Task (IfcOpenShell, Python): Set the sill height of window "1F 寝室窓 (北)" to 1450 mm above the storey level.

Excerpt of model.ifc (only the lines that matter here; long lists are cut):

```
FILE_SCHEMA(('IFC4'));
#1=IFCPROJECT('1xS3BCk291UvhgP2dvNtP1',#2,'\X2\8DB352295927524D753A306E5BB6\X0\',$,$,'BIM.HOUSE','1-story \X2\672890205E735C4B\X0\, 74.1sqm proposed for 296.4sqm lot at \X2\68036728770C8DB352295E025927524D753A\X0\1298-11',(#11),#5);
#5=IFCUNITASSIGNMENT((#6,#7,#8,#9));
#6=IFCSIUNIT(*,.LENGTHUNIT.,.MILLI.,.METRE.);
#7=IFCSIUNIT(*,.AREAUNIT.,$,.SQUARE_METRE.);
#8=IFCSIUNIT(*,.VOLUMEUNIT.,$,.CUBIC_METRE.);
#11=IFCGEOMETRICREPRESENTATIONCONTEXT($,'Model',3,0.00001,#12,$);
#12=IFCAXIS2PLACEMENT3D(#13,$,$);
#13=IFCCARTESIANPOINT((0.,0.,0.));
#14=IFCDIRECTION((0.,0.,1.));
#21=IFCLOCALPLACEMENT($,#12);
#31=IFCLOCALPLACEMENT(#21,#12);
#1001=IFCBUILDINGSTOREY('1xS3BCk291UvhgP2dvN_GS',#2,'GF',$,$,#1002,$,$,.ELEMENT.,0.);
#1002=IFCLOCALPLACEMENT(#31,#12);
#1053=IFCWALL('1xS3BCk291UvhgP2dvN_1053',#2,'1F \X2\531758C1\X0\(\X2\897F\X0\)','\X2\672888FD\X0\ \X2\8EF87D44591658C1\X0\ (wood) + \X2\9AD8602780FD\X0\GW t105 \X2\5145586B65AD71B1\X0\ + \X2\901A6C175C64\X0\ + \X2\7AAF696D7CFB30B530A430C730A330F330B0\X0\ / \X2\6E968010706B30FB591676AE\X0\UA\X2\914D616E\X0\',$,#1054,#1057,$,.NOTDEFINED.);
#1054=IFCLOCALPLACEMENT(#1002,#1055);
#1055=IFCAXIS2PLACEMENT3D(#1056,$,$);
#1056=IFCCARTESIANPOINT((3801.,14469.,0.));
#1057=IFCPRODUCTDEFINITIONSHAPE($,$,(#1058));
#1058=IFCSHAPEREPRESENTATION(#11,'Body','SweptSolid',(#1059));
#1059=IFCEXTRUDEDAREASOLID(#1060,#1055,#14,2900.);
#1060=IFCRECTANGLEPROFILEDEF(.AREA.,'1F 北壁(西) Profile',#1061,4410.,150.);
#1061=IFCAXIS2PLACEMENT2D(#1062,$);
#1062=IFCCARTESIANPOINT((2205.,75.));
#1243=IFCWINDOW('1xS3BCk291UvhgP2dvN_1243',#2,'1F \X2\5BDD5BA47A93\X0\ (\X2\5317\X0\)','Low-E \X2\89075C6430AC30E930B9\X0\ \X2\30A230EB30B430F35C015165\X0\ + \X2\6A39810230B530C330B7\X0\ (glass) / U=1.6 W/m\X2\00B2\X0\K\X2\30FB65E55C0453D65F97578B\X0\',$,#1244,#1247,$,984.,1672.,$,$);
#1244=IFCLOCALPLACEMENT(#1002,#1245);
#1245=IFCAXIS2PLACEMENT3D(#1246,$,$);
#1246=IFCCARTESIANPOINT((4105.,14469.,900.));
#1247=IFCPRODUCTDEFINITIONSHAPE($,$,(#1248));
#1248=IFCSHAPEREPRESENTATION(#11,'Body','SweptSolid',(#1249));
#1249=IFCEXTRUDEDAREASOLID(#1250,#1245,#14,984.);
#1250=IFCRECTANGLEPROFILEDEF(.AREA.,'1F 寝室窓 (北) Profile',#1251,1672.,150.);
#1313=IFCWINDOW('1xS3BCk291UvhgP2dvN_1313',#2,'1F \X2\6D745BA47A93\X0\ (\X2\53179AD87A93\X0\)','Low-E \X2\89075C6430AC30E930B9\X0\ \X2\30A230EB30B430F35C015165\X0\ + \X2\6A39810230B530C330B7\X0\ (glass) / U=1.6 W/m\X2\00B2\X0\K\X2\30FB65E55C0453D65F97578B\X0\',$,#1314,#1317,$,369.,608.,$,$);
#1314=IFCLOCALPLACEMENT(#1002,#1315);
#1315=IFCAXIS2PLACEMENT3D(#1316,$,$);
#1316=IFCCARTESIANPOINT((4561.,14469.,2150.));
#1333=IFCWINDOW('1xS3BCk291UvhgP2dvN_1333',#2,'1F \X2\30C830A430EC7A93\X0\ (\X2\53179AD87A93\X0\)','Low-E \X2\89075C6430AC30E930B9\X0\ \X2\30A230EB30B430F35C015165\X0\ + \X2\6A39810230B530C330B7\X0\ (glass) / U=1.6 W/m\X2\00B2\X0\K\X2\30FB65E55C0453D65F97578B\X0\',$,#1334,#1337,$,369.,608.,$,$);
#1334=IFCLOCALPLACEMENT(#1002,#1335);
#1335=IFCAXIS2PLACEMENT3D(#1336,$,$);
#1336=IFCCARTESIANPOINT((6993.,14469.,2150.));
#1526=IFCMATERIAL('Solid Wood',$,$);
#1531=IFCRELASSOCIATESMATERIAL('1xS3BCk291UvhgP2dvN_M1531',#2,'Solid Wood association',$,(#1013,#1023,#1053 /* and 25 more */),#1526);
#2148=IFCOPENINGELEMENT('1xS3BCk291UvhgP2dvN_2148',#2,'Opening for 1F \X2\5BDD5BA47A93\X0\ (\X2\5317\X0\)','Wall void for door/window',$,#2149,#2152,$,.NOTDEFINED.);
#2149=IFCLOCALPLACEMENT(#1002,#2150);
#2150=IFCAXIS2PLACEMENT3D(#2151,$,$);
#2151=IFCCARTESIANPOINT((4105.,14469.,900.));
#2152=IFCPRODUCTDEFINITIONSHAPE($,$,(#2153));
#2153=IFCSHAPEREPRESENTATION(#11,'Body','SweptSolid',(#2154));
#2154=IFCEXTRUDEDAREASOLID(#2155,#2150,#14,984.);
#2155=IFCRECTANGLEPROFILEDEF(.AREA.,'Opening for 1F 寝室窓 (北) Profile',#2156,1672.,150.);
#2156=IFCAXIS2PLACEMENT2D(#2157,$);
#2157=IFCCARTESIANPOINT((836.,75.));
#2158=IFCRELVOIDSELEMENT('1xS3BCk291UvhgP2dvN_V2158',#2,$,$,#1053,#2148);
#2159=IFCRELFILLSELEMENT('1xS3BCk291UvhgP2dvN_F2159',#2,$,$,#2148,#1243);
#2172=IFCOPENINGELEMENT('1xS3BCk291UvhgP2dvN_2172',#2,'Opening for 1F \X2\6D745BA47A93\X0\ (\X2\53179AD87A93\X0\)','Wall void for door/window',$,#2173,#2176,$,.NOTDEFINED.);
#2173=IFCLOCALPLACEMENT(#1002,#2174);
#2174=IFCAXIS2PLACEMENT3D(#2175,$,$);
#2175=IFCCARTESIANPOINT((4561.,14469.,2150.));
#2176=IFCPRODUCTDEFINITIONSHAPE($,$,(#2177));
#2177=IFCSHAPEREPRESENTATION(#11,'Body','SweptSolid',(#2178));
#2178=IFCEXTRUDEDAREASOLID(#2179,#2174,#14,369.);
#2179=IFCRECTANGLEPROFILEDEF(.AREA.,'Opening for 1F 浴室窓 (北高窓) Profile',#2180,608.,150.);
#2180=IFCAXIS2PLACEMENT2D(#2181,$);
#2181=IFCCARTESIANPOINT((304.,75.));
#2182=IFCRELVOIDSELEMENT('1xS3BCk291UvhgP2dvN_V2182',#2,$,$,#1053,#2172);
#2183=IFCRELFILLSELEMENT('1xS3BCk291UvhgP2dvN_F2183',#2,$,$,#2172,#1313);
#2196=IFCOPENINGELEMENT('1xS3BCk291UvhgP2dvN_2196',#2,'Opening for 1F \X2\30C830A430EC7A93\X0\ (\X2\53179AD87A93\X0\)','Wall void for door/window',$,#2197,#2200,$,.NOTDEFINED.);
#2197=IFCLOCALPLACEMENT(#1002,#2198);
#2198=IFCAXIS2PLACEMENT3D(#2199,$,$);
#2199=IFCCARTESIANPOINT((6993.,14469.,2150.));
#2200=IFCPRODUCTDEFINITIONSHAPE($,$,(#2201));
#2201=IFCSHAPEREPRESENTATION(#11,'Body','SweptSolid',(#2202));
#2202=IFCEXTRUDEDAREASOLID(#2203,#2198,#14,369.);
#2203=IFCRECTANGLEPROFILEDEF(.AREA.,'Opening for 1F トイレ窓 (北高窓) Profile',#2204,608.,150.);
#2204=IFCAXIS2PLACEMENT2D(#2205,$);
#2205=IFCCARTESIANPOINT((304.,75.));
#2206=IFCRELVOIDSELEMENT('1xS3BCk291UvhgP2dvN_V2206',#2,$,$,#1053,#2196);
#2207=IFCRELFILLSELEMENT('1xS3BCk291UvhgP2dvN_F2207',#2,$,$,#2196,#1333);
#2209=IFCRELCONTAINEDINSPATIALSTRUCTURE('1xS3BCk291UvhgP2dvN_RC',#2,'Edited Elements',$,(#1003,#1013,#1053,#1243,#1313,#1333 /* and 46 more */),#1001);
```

```python
import numpy as np
import ifcopenshell
import ifcopenshell.api.geometry
import ifcopenshell.geom
import ifcopenshell.util.element
import ifcopenshell.util.placement
import ifcopenshell.util.shape
import ifcopenshell.util.unit

model = ifcopenshell.open("model.ifc")
unit_scale = ifcopenshell.util.unit.calculate_unit_scale(model)

window = model.by_id(1243)
opening = window.FillsVoids[0].RelatingOpeningElement
storey = ifcopenshell.util.element.get_container(window, ifc_class="IfcBuildingStorey")
level = ifcopenshell.util.placement.get_local_placement(storey.ObjectPlacement)[2, 3]

# The opening's origin need not be at the sill, so measure its lowest point.
shape = ifcopenshell.geom.create_shape(ifcopenshell.geom.settings(), opening)
bottom = ifcopenshell.util.shape.get_shape_bottom_elevation(shape, shape.geometry) / unit_scale
dz = level + 1.45 / unit_scale - bottom

shift = np.array([0.0, 0.0, dz])
# The window is not placed relative to its opening, so move both.
for product in (opening, window):
    matrix = ifcopenshell.util.placement.get_local_placement(product.ObjectPlacement)
    matrix[:3, 3] += shift
    ifcopenshell.api.geometry.edit_object_placement(model, product=product, matrix=matrix, is_si=False)

print(f"moved by {dz * unit_scale:+.3f} m")

model.write("model-out.ifc")
```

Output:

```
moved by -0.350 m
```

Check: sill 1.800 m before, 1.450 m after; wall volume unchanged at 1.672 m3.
